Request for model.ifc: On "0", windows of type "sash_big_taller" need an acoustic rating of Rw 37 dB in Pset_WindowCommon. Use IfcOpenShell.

First a look at what the model holds.

```python
import ifcopenshell
import ifcopenshell.util.element

model = ifcopenshell.open("model.ifc")
print(model.schema)
storey = next(s for s in model.by_type("IfcBuildingStorey") if s.Name == "0")
windows = [e for e in ifcopenshell.util.element.get_decomposition(storey) if e.is_a("IfcWindow")]
seen = {}
for e in windows:
    element_type = ifcopenshell.util.element.get_type(e)
    key = (element_type.Name if element_type != e and element_type else None, ifcopenshell.util.element.get_pset(e, "Pset_WindowCommon", "AcousticRating"))
    seen[key] = seen.get(key, 0) + 1
for (name, value), count in sorted(seen.items(), key=str):
    print(count, "x", name, "|", value)
```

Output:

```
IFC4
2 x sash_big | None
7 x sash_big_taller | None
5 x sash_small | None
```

```python
import ifcopenshell
import ifcopenshell.api.pset
import ifcopenshell.util.element

model = ifcopenshell.open("model.ifc")

storey = next(s for s in model.by_type("IfcBuildingStorey") if s.Name == "0")
windows = [e for e in ifcopenshell.util.element.get_decomposition(storey) if e.is_a("IfcWindow")]

count = 0
for e in windows:
    element_type = ifcopenshell.util.element.get_type(e)
    if element_type in (None, e) or element_type.Name != "sash_big_taller":
        continue
    # add_pset returns the element's existing set when there is one.
    pset = ifcopenshell.api.pset.add_pset(model, product=e, name="Pset_WindowCommon")
    ifcopenshell.api.pset.edit_pset(model, pset=pset, properties={"AcousticRating": "Rw 37 dB"})
    count += 1

print(count, "windows updated")

model.write("model_updated.ifc")
```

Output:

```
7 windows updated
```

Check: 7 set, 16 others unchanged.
